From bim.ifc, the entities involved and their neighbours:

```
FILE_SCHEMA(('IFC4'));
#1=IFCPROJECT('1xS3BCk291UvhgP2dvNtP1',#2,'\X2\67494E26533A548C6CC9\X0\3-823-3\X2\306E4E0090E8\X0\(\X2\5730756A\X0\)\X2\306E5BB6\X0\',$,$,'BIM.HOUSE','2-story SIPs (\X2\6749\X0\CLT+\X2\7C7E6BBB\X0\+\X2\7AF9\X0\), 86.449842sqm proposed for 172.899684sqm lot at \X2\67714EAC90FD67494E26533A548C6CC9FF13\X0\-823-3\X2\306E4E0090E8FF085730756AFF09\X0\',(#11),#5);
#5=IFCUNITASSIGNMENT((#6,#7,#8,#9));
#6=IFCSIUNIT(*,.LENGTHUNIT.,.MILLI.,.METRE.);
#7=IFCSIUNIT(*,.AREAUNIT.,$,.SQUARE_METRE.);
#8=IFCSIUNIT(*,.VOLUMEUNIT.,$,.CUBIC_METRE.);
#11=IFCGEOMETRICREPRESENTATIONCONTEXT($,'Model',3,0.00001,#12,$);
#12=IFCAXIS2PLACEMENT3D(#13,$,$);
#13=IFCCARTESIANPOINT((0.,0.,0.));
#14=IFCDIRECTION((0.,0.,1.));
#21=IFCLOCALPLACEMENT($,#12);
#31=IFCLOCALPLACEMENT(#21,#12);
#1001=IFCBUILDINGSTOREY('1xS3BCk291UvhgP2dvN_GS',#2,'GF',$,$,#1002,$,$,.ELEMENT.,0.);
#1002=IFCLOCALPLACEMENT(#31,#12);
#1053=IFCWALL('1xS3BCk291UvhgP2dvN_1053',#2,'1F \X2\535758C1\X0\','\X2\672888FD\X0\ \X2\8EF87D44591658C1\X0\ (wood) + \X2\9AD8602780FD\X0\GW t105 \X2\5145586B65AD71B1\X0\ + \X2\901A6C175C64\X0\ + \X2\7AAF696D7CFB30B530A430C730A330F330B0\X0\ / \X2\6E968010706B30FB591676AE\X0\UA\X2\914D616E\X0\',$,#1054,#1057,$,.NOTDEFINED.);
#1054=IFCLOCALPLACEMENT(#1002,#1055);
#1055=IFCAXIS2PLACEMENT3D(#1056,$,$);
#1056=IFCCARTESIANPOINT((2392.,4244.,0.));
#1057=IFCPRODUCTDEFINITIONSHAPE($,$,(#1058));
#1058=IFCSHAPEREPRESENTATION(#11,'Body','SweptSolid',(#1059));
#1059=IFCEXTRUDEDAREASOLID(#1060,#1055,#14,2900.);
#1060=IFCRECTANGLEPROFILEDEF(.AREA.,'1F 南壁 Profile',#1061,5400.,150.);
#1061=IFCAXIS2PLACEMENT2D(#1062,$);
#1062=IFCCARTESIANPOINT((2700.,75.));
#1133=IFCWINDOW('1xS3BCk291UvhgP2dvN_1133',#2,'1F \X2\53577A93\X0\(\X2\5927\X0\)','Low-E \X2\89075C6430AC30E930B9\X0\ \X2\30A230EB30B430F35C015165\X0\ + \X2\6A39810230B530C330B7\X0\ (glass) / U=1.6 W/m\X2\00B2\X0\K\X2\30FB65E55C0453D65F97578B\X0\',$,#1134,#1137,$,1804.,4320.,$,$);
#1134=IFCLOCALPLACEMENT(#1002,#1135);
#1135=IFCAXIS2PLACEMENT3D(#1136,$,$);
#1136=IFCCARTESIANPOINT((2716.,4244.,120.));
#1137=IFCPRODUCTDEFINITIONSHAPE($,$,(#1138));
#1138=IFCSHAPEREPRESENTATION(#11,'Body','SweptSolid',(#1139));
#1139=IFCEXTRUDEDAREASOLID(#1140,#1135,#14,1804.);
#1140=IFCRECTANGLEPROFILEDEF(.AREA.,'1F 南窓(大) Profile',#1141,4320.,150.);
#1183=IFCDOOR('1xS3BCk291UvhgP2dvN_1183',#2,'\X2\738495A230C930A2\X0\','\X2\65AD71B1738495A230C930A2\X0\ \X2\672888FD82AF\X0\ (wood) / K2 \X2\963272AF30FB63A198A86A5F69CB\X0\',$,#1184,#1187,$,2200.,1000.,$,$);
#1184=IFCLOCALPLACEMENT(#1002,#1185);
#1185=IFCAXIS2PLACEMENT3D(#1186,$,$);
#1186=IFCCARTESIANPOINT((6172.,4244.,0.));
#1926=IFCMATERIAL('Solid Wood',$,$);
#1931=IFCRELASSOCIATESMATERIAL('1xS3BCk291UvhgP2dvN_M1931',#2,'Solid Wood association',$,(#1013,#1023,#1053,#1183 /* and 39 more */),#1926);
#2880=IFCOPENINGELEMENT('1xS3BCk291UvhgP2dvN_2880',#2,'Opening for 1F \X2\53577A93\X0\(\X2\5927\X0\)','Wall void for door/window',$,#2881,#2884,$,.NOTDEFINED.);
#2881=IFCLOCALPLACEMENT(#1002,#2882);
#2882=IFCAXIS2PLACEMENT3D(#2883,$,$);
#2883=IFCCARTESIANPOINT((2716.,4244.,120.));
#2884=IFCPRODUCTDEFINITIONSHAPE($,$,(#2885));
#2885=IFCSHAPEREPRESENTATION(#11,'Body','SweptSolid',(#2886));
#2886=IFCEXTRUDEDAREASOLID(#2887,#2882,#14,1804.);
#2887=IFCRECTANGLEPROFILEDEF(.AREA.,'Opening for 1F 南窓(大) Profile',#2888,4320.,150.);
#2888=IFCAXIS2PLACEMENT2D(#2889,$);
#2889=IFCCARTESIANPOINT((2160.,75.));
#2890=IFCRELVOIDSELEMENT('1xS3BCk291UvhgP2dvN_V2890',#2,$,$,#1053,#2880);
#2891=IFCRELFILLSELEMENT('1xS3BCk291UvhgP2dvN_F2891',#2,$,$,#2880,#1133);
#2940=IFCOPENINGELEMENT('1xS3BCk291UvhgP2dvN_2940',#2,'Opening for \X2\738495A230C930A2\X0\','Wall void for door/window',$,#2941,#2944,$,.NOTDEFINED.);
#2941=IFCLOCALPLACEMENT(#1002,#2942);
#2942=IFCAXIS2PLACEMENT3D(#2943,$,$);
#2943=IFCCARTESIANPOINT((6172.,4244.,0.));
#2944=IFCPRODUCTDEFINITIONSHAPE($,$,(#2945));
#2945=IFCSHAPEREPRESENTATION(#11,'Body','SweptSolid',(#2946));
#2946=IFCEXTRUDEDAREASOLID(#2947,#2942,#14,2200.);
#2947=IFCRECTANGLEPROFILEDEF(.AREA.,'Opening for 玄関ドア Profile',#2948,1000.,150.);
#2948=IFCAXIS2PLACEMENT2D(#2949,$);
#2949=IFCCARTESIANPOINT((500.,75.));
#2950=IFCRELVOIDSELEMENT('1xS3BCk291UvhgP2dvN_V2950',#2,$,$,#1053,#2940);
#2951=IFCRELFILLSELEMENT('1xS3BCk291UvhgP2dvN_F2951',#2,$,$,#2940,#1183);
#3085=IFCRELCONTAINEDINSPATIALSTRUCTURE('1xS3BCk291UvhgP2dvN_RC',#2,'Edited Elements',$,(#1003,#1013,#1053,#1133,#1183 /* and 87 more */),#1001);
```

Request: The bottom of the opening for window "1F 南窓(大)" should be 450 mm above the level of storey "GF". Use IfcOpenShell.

```python
import numpy as np
import ifcopenshell
import ifcopenshell.api.geometry
import ifcopenshell.geom
import ifcopenshell.util.element
import ifcopenshell.util.placement
import ifcopenshell.util.shape
import ifcopenshell.util.unit

model = ifcopenshell.open("bim.ifc")
unit_scale = ifcopenshell.util.unit.calculate_unit_scale(model)

window = model.by_guid("1xS3BCk291UvhgP2dvN_1133")
opening = window.FillsVoids[0].RelatingOpeningElement
storey = ifcopenshell.util.element.get_container(window, ifc_class="IfcBuildingStorey")
level = ifcopenshell.util.placement.get_local_placement(storey.ObjectPlacement)[2, 3]

# The opening's origin need not be at the sill, so measure its lowest point.
shape = ifcopenshell.geom.create_shape(ifcopenshell.geom.settings(), opening)
bottom = ifcopenshell.util.shape.get_shape_bottom_elevation(shape, shape.geometry) / unit_scale
dz = level + 450.0 - bottom

shift = np.array([0.0, 0.0, dz])
# The window is not placed relative to its opening, so move both.
for product in (opening, window):
    matrix = ifcopenshell.util.placement.get_local_placement(product.ObjectPlacement)
    matrix[:3, 3] += shift
    ifcopenshell.api.geometry.edit_object_placement(model, product=product, matrix=matrix, is_si=False)

print(f"moved by {dz * unit_scale:+.3f} m")

model.write("bim_v2.ifc")
```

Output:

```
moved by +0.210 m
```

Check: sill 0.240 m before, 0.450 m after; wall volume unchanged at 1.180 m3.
